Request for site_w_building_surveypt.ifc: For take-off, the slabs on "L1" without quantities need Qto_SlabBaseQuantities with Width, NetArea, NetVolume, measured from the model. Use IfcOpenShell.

First a look at what the model holds.

```python
import ifcopenshell
import ifcopenshell.util.element
import ifcopenshell.util.unit

model = ifcopenshell.open("site_w_building_surveypt.ifc")
print(model.schema)
for unit_type in ("LENGTHUNIT", "AREAUNIT", "VOLUMEUNIT"):
    print(unit_type, ifcopenshell.util.unit.calculate_unit_scale(model, unit_type))
storey = next(s for s in model.by_type("IfcBuildingStorey") if s.Name == "L1")
slabs = [e for e in ifcopenshell.util.element.get_decomposition(storey) if e.is_a("IfcSlab")]
for e in sorted(slabs, key=lambda e: e.id()):
    print(e.id(), e.is_a(), e.Name, list(ifcopenshell.util.element.get_psets(e, qtos_only=True)), sep=" | ")
```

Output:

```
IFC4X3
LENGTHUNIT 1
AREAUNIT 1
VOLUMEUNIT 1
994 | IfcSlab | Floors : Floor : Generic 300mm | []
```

```python
import ifcopenshell
import ifcopenshell.api.pset
import ifcopenshell.geom
import ifcopenshell.util.element
import ifcopenshell.util.shape
import ifcopenshell.util.unit

model = ifcopenshell.open("site_w_building_surveypt.ifc")
unit_scale = ifcopenshell.util.unit.calculate_unit_scale(model)
area_scale = ifcopenshell.util.unit.calculate_unit_scale(model, "AREAUNIT")
volume_scale = ifcopenshell.util.unit.calculate_unit_scale(model, "VOLUMEUNIT")
settings = ifcopenshell.geom.settings()

storey = next(s for s in model.by_type("IfcBuildingStorey") if s.Name == "L1")
slabs = [e for e in ifcopenshell.util.element.get_decomposition(storey) if e.is_a("IfcSlab")]

for e in sorted(slabs, key=lambda e: e.id()):
    if ifcopenshell.util.element.get_psets(e, qtos_only=True, should_inherit=False):
        continue
    # Geometry comes back in metres, in the element's own axes.
    shape = ifcopenshell.geom.create_shape(settings, e)
    values = {
        "Width": ifcopenshell.util.shape.get_z(shape.geometry) / unit_scale,
        "NetArea": ifcopenshell.util.shape.get_footprint_area(shape.geometry) / area_scale,
        "NetVolume": ifcopenshell.util.shape.get_volume(shape.geometry) / volume_scale,
    }
    qto = ifcopenshell.api.pset.add_qto(model, product=e, name="Qto_SlabBaseQuantities")
    ifcopenshell.api.pset.edit_qto(model, qto=qto, properties=values)
    print(e.id(), {k: round(v, 3) for k, v in values.items()})

model.write("site_w_building_surveypt_rev.ifc")
```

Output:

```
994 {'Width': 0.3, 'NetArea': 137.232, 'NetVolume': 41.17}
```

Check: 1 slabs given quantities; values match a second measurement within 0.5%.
